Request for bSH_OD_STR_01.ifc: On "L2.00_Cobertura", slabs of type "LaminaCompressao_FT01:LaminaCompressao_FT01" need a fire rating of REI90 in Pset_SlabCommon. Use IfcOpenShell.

First a look at what the model holds.

```python
import ifcopenshell
import ifcopenshell.util.element

model = ifcopenshell.open("bSH_OD_STR_01.ifc")
print(model.schema)
storey = next(s for s in model.by_type("IfcBuildingStorey") if s.Name == "L2.00_Cobertura")
slabs = [e for e in ifcopenshell.util.element.get_decomposition(storey) if e.is_a("IfcSlab")]
seen = {}
for e in slabs:
    element_type = ifcopenshell.util.element.get_type(e)
    key = (element_type.Name if element_type != e and element_type else None, ifcopenshell.util.element.get_pset(e, "Pset_SlabCommon", "FireRating"))
    seen[key] = seen.get(key, 0) + 1
for (name, value), count in sorted(seen.items(), key=str):
    print(count, "x", name, "|", value)
```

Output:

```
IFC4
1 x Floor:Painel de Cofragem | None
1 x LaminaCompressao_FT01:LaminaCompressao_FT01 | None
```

```python
import ifcopenshell
import ifcopenshell.api.pset
import ifcopenshell.util.element

model = ifcopenshell.open("bSH_OD_STR_01.ifc")

storey = next(s for s in model.by_type("IfcBuildingStorey") if s.Name == "L2.00_Cobertura")
slabs = [e for e in ifcopenshell.util.element.get_decomposition(storey) if e.is_a("IfcSlab")]

count = 0
for e in slabs:
    element_type = ifcopenshell.util.element.get_type(e)
    if element_type in (None, e) or element_type.Name != "LaminaCompressao_FT01:LaminaCompressao_FT01":
        continue
    # add_pset returns the element's existing set when there is one.
    pset = ifcopenshell.api.pset.add_pset(model, product=e, name="Pset_SlabCommon")
    ifcopenshell.api.pset.edit_pset(model, pset=pset, properties={"FireRating": "REI90"})
    count += 1

print(count, "slabs updated")

model.write("bSH_OD_STR_01-out.ifc")
```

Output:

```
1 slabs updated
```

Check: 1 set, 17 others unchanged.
